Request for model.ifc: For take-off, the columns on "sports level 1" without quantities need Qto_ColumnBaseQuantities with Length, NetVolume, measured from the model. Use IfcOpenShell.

First a look at what the model holds.

```python
import ifcopenshell
import ifcopenshell.util.element
import ifcopenshell.util.unit

model = ifcopenshell.open("model.ifc")
print(model.schema)
for unit_type in ("LENGTHUNIT", "AREAUNIT", "VOLUMEUNIT"):
    print(unit_type, ifcopenshell.util.unit.calculate_unit_scale(model, unit_type))
storey = next(s for s in model.by_type("IfcBuildingStorey") if s.Name == "sports level 1")
columns = [e for e in ifcopenshell.util.element.get_decomposition(storey) if e.is_a("IfcColumn")]
for e in sorted(columns, key=lambda e: e.id()):
    print(e.id(), e.is_a(), e.Name, list(ifcopenshell.util.element.get_psets(e, qtos_only=True)), sep=" | ")
```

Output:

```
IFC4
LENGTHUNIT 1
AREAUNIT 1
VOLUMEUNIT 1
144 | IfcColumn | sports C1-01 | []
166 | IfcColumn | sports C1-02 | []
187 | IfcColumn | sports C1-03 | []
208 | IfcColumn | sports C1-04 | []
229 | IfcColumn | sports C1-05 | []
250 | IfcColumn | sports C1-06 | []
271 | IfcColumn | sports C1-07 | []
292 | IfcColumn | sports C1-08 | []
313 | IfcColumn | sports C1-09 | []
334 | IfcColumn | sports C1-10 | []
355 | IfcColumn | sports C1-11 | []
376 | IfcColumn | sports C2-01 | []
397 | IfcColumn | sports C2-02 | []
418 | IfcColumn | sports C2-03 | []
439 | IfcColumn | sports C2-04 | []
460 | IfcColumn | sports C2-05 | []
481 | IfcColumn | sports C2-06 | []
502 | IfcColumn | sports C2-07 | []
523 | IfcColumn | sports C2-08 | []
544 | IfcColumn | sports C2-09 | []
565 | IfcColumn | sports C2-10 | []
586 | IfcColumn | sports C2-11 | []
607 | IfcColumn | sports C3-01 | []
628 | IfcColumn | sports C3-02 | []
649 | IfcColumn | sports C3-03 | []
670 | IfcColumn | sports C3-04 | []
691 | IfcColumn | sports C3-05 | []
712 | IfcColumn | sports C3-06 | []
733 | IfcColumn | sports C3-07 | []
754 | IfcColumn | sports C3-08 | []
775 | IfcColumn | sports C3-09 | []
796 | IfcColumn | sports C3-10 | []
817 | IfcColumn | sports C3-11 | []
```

```python
import ifcopenshell
import ifcopenshell.api.pset
import ifcopenshell.geom
import ifcopenshell.util.element
import ifcopenshell.util.shape
import ifcopenshell.util.unit

model = ifcopenshell.open("model.ifc")
unit_scale = ifcopenshell.util.unit.calculate_unit_scale(model)
volume_scale = ifcopenshell.util.unit.calculate_unit_scale(model, "VOLUMEUNIT")
settings = ifcopenshell.geom.settings()

storey = next(s for s in model.by_type("IfcBuildingStorey") if s.Name == "sports level 1")
columns = [e for e in ifcopenshell.util.element.get_decomposition(storey) if e.is_a("IfcColumn")]

for e in sorted(columns, key=lambda e: e.id()):
    if ifcopenshell.util.element.get_psets(e, qtos_only=True, should_inherit=False):
        continue
    # Geometry comes back in metres, in the element's own axes.
    shape = ifcopenshell.geom.create_shape(settings, e)
    values = {
        "Length": ifcopenshell.util.shape.get_z(shape.geometry) / unit_scale,
        "NetVolume": ifcopenshell.util.shape.get_volume(shape.geometry) / volume_scale,
    }
    qto = ifcopenshell.api.pset.add_qto(model, product=e, name="Qto_ColumnBaseQuantities")
    ifcopenshell.api.pset.edit_qto(model, qto=qto, properties=values)
    print(e.id(), {k: round(v, 3) for k, v in values.items()})

model.write("model_rev.ifc")
```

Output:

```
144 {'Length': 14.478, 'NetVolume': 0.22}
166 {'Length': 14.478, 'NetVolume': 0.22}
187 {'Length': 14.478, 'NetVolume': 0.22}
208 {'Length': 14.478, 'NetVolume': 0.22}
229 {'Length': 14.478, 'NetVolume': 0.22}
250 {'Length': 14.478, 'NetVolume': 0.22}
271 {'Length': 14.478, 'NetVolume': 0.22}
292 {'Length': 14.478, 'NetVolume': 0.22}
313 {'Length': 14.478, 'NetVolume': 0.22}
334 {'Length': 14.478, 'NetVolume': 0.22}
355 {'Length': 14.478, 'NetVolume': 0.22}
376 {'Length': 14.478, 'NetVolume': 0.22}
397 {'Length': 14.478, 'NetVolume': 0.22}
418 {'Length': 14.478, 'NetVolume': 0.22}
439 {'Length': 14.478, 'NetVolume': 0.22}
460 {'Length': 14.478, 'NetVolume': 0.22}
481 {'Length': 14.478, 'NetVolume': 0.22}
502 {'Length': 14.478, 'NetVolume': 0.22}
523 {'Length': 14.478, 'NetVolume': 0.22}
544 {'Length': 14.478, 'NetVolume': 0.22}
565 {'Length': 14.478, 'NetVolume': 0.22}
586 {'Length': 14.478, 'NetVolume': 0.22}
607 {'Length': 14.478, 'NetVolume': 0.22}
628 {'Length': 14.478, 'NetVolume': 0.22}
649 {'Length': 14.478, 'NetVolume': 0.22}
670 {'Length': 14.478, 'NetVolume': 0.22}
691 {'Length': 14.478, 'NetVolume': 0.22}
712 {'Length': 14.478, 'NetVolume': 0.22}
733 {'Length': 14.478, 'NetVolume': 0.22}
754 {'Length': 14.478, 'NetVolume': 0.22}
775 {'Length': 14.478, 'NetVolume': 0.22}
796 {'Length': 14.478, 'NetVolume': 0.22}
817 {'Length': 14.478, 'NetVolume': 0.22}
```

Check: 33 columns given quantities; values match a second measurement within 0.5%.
